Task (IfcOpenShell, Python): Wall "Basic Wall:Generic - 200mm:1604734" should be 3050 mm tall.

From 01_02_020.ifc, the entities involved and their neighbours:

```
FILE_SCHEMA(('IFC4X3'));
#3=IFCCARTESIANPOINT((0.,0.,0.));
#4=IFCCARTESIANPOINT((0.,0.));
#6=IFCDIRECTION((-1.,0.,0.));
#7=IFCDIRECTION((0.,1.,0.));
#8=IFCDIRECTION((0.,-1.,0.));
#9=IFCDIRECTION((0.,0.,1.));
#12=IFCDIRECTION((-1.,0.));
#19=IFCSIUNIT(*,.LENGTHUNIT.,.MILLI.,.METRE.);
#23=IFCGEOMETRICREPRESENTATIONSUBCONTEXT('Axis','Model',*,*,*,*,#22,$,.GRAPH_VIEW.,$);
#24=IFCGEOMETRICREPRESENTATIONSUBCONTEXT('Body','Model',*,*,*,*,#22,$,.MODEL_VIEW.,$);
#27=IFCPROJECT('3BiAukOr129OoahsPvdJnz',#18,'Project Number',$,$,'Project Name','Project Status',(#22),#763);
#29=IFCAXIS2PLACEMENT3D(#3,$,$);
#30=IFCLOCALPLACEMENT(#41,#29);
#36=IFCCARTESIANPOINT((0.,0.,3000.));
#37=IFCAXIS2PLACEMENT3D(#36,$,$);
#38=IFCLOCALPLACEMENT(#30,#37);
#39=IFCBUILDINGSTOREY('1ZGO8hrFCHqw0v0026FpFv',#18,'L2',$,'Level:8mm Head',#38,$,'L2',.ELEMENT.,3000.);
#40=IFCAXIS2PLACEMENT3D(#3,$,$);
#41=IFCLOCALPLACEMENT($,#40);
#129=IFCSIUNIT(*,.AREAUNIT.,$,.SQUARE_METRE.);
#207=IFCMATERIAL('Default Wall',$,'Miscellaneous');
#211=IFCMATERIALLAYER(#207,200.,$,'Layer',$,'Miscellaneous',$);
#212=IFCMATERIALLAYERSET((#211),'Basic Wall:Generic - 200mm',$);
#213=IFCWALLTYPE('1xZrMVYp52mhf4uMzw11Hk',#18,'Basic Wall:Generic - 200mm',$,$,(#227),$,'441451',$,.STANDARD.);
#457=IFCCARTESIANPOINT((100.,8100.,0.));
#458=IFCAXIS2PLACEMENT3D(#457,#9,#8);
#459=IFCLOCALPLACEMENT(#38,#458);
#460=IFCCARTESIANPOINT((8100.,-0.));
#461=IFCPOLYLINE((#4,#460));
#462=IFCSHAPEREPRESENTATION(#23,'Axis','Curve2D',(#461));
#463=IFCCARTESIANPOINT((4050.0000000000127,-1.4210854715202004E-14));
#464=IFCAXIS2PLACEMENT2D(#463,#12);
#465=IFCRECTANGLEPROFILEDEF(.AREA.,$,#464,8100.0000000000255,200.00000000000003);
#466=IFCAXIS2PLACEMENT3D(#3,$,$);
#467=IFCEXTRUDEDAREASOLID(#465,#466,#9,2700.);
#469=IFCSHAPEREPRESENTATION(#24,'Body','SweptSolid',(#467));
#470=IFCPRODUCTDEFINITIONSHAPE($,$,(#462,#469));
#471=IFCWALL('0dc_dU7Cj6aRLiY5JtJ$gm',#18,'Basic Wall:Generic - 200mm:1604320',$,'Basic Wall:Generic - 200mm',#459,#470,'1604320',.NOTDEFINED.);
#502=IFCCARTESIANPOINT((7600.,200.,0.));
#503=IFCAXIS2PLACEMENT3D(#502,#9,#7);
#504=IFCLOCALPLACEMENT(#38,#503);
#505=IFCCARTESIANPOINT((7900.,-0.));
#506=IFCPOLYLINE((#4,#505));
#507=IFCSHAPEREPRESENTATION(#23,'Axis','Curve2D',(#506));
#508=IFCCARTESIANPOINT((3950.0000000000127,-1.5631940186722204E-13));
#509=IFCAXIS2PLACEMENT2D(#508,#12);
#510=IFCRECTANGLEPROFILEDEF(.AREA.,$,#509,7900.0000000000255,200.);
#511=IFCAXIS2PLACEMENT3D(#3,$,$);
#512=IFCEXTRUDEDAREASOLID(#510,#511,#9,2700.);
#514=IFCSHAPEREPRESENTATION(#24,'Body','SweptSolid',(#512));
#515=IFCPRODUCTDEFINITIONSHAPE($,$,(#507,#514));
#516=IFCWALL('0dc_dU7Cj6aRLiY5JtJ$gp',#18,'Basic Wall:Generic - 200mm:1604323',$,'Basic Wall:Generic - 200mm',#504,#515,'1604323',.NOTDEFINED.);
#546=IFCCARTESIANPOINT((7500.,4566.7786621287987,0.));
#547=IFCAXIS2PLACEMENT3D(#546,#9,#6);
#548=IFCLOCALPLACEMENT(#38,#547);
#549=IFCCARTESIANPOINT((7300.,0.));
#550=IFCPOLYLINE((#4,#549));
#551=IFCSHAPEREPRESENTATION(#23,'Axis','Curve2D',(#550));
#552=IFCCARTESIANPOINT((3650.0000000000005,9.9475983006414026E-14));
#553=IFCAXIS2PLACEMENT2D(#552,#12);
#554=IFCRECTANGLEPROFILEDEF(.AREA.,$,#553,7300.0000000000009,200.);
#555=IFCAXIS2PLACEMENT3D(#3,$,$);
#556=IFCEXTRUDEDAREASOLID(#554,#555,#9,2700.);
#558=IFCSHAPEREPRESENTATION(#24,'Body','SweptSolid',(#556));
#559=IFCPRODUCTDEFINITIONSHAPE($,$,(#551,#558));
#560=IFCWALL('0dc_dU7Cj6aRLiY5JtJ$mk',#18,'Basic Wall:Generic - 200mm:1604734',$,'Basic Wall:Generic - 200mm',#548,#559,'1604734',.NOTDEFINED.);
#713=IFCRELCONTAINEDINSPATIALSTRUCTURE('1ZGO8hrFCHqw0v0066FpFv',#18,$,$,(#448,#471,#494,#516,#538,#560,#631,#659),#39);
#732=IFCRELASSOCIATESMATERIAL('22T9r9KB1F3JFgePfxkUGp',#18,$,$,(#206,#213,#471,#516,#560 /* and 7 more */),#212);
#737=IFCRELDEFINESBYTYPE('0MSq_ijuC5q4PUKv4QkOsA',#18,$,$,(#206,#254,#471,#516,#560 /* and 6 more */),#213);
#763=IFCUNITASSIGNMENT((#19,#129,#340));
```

```python
import ifcopenshell
import ifcopenshell.geom
import ifcopenshell.util.representation
import ifcopenshell.util.shape
import ifcopenshell.util.unit

model = ifcopenshell.open("01_02_020.ifc")
unit_scale = ifcopenshell.util.unit.calculate_unit_scale(model)
settings = ifcopenshell.geom.settings()


def volume(element):
    """Net volume in cubic metres, openings subtracted."""
    shape = ifcopenshell.geom.create_shape(settings, element)
    return ifcopenshell.util.shape.get_volume(shape.geometry)


wall = model.by_guid("0dc_dU7Cj6aRLiY5JtJ$mk")
before = volume(wall)

body = ifcopenshell.util.representation.get_representation(wall, "Model", "Body")
solid = body.Items[0]
old_height = solid.Depth
solid.Depth = 3.05 / unit_scale
after = volume(wall)

print(f"height {old_height:g} -> {solid.Depth:g}, volume {before:.3f} -> {after:.3f} m3")

model.write("01_02_020_updated.ifc")
```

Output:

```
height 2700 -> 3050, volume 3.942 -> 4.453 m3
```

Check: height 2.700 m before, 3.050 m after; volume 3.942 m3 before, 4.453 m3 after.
